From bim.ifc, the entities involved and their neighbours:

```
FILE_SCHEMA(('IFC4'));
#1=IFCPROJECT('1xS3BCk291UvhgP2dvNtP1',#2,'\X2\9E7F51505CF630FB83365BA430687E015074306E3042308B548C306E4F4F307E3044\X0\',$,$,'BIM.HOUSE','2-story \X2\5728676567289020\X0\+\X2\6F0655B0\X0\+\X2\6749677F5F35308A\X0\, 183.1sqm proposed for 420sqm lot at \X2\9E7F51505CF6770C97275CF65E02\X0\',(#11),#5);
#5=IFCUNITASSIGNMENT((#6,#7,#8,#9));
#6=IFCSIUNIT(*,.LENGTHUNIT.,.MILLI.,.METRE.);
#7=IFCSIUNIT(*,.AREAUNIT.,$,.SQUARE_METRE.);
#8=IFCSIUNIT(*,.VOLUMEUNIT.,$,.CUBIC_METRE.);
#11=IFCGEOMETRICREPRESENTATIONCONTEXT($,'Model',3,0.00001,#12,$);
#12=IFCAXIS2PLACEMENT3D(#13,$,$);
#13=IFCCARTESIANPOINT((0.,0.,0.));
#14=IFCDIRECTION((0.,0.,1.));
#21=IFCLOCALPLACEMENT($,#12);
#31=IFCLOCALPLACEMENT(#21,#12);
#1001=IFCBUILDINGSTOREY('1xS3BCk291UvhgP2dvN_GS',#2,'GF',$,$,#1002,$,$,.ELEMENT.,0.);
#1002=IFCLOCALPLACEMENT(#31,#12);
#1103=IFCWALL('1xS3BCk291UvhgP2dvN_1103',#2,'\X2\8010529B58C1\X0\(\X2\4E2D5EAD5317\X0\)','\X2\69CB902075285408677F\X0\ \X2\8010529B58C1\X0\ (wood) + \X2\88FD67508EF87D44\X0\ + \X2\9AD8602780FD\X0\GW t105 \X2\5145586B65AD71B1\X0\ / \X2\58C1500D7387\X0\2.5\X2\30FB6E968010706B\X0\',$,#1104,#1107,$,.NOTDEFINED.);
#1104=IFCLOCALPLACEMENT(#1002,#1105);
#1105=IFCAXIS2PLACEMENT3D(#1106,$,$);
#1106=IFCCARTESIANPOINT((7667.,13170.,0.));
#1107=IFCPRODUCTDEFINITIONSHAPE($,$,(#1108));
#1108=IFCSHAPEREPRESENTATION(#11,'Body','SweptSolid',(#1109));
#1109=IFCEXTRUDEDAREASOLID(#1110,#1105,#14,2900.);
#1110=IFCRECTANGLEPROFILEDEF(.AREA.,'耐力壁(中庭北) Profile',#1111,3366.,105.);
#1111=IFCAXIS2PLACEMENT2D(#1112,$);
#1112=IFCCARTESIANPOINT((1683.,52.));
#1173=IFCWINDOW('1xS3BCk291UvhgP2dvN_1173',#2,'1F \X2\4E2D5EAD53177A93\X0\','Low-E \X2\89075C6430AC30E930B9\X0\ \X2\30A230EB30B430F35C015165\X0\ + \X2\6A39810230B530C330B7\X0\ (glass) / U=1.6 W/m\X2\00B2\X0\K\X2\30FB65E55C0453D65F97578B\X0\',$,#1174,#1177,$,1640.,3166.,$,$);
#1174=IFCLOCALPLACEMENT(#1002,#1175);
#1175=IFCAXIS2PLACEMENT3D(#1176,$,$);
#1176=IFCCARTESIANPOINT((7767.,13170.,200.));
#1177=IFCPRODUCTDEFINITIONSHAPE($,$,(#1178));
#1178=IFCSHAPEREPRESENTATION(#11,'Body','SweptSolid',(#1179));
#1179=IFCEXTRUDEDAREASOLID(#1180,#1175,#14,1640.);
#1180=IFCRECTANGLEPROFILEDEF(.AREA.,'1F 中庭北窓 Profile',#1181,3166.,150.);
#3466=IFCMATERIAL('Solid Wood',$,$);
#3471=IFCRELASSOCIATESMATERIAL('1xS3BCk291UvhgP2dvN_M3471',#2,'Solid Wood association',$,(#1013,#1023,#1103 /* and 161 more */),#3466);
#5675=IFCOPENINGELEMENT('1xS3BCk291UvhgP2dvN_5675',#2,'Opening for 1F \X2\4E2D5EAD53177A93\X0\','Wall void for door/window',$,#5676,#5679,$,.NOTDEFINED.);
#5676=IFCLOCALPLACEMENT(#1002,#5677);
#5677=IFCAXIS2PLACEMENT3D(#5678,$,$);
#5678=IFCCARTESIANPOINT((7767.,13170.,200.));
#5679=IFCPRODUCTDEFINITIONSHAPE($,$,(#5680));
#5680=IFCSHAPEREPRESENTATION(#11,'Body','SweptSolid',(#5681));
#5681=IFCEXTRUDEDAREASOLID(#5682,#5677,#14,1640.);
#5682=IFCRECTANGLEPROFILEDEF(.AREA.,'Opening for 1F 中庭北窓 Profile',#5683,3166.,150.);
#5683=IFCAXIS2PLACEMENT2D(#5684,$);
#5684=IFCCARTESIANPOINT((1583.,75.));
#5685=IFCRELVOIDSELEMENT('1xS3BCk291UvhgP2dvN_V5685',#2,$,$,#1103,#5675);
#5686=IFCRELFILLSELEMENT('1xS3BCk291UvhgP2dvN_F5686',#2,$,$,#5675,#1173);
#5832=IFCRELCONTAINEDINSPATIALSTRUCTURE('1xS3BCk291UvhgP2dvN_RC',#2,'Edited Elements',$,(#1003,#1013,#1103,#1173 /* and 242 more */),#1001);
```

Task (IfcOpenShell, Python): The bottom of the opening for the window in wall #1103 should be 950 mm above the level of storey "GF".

```python
import numpy as np
import ifcopenshell
import ifcopenshell.api.geometry
import ifcopenshell.geom
import ifcopenshell.util.element
import ifcopenshell.util.placement
import ifcopenshell.util.shape
import ifcopenshell.util.unit

model = ifcopenshell.open("bim.ifc")
unit_scale = ifcopenshell.util.unit.calculate_unit_scale(model)

window = model.by_id(1173)
opening = window.FillsVoids[0].RelatingOpeningElement
storey = ifcopenshell.util.element.get_container(window, ifc_class="IfcBuildingStorey")
level = ifcopenshell.util.placement.get_local_placement(storey.ObjectPlacement)[2, 3]

# The opening's origin need not be at the sill, so measure its lowest point.
shape = ifcopenshell.geom.create_shape(ifcopenshell.geom.settings(), opening)
bottom = ifcopenshell.util.shape.get_shape_bottom_elevation(shape, shape.geometry) / unit_scale
dz = level + 950.0 - bottom

shift = np.array([0.0, 0.0, dz])
# The window is not placed relative to its opening, so move both.
for product in (opening, window):
    matrix = ifcopenshell.util.placement.get_local_placement(product.ObjectPlacement)
    matrix[:3, 3] += shift
    ifcopenshell.api.geometry.edit_object_placement(model, product=product, matrix=matrix, is_si=False)

print(f"moved by {dz * unit_scale:+.3f} m")

model.write("bim_v2.ifc")
```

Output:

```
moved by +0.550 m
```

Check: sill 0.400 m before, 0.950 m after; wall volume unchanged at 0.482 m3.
